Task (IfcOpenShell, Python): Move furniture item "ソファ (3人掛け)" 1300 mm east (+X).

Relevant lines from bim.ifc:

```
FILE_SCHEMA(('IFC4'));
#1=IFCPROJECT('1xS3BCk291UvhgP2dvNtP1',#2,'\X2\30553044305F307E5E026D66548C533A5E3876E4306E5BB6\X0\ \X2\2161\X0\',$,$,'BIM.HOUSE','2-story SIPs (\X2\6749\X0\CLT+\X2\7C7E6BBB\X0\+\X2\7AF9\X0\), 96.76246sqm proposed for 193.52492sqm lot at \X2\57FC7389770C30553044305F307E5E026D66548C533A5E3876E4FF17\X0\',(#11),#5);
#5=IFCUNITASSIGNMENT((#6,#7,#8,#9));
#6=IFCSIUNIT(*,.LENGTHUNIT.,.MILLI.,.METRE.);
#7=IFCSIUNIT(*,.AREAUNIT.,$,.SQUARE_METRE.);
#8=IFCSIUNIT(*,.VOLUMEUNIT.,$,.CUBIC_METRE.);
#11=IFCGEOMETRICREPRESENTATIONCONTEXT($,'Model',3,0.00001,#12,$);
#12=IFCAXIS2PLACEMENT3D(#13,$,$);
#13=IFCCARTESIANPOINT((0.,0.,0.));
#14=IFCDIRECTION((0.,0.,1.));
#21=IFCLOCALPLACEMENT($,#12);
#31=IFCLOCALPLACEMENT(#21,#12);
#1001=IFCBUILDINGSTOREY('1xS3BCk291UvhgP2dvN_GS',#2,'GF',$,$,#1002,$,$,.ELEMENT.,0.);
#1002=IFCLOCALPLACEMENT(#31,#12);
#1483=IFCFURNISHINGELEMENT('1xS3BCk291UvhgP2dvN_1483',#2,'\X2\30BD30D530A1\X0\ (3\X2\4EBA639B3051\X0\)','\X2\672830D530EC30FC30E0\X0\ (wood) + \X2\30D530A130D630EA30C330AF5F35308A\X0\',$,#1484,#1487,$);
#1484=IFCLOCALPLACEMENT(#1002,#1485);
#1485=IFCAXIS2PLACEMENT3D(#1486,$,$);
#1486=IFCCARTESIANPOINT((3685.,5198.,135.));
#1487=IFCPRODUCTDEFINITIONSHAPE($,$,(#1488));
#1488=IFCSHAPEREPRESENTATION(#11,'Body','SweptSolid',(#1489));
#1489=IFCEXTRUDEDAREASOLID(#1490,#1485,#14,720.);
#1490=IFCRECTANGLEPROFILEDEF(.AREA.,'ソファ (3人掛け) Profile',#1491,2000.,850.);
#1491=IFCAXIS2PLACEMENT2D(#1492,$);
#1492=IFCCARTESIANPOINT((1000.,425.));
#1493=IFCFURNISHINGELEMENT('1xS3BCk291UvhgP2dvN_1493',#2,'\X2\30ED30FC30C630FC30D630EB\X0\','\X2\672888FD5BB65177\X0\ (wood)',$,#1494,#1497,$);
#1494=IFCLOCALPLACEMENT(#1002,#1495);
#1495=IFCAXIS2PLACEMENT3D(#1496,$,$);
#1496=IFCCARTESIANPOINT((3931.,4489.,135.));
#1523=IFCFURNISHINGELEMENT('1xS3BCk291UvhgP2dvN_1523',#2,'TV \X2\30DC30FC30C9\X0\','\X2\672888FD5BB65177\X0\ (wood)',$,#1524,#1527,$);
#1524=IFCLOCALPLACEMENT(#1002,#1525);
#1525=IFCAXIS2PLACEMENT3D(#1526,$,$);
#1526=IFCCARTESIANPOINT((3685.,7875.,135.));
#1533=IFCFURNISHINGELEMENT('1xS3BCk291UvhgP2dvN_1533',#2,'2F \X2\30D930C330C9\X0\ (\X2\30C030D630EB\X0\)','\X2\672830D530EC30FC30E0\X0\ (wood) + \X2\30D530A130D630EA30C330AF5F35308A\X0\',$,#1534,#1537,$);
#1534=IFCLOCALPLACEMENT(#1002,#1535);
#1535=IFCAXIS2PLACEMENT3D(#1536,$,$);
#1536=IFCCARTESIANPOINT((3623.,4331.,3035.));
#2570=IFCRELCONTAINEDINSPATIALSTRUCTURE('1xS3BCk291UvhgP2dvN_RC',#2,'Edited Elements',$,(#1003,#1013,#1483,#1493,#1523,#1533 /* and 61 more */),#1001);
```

```python
import ifcopenshell
import ifcopenshell.api.geometry
import ifcopenshell.util.placement
import ifcopenshell.util.unit

model = ifcopenshell.open("bim.ifc")
unit_scale = ifcopenshell.util.unit.calculate_unit_scale(model)

item = model.by_guid("1xS3BCk291UvhgP2dvN_1483")
matrix = ifcopenshell.util.placement.get_local_placement(item.ObjectPlacement)
matrix[0, 3] += 1.3 / unit_scale
ifcopenshell.api.geometry.edit_object_placement(model, product=item, matrix=matrix, is_si=False)

print(ifcopenshell.util.placement.get_local_placement(item.ObjectPlacement).round(3) + 0.0)

model.write("bim-out.ifc")
```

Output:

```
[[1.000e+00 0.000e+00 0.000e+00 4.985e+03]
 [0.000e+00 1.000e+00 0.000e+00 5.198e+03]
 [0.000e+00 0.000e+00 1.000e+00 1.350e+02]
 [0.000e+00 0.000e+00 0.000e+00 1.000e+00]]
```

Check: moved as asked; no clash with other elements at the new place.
